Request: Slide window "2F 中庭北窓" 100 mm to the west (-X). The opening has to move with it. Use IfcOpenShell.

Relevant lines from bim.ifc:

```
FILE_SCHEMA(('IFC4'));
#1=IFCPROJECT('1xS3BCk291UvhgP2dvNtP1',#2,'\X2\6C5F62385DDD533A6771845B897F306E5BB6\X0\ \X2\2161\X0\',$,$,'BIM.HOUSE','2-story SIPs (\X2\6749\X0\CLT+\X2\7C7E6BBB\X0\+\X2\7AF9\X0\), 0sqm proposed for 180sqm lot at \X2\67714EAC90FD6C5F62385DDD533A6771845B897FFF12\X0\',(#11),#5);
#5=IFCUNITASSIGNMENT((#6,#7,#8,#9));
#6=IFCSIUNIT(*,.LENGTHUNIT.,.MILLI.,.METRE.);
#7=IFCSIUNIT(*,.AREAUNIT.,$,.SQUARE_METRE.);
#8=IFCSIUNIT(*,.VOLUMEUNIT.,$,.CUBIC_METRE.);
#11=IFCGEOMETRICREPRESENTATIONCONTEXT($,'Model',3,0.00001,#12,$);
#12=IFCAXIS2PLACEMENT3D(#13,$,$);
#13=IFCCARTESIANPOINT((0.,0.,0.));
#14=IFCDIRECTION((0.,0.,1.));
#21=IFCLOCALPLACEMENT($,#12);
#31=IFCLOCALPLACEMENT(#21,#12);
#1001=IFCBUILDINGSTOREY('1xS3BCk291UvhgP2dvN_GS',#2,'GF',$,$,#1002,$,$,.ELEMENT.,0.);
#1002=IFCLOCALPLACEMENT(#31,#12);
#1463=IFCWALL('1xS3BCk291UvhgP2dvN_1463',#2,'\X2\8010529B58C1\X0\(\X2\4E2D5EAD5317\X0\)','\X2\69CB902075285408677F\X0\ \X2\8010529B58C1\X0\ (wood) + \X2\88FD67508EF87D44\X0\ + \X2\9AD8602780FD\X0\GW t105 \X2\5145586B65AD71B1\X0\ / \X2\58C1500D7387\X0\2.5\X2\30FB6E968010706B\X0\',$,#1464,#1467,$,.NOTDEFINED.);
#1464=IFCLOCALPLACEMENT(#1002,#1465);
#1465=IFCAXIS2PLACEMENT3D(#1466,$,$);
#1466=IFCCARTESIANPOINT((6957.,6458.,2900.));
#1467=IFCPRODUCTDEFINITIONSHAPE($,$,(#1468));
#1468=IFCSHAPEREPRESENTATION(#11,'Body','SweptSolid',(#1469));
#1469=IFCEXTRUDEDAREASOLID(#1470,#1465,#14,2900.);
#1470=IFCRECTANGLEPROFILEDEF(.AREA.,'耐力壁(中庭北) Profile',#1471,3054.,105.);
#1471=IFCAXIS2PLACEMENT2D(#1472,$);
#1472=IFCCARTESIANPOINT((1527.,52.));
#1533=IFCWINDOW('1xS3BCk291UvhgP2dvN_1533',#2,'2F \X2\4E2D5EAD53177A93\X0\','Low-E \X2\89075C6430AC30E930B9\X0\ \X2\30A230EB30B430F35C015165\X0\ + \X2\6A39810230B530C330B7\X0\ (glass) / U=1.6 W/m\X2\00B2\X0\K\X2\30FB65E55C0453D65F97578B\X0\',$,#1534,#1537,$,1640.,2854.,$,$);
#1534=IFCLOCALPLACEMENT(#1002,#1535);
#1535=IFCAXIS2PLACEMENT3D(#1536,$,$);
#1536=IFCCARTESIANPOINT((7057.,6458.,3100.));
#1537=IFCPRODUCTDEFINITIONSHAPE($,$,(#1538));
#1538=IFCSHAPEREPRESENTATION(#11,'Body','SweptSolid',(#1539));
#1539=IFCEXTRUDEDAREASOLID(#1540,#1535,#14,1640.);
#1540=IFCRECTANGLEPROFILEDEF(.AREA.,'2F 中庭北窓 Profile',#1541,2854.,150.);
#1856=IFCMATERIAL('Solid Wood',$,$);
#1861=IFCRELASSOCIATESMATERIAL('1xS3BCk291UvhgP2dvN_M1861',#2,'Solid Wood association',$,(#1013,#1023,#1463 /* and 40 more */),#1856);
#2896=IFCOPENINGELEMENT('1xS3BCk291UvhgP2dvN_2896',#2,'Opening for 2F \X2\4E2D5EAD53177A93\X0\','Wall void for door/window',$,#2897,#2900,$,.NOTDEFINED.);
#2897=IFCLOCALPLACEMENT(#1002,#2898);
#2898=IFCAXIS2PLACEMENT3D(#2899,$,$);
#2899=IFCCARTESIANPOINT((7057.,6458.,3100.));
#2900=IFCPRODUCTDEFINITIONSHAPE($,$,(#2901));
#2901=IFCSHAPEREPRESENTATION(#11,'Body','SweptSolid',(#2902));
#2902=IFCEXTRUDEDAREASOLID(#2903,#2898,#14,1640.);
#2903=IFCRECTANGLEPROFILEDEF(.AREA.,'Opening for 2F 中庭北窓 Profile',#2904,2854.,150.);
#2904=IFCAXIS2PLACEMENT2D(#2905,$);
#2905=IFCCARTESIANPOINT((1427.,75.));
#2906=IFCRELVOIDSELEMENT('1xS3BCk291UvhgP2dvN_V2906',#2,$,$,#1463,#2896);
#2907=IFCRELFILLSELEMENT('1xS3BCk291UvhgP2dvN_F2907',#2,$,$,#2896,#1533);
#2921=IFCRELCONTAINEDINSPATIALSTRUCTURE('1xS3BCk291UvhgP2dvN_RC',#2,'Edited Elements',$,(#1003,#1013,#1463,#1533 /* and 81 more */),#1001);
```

```python
import ifcopenshell
import ifcopenshell.api.geometry
import ifcopenshell.util.placement

model = ifcopenshell.open("bim.ifc")

window = model.by_guid("1xS3BCk291UvhgP2dvN_1533")
opening = window.FillsVoids[0].RelatingOpeningElement
wall = opening.VoidsElements[0].RelatingBuildingElement

wall_matrix = ifcopenshell.util.placement.get_local_placement(wall.ObjectPlacement)
shift = wall_matrix[:3, 0] * -100.0
before = ifcopenshell.util.placement.get_local_placement(window.ObjectPlacement)[:3, 3].copy()

# The window is not placed relative to its opening, so move both.
for product in (opening, window):
    matrix = ifcopenshell.util.placement.get_local_placement(product.ObjectPlacement)
    matrix[:3, 3] += shift
    ifcopenshell.api.geometry.edit_object_placement(model, product=product, matrix=matrix, is_si=False)

after = ifcopenshell.util.placement.get_local_placement(window.ObjectPlacement)[:3, 3]
print("window moved by", (after - before).round(3) + 0.0)

model.write("bim_v2.ifc")
```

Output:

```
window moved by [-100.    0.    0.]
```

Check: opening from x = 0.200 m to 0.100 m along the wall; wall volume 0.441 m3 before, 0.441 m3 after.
